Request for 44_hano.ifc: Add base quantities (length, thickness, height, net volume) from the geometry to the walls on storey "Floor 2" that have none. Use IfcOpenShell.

First a look at what the model holds.

```python
import ifcopenshell
import ifcopenshell.util.element
import ifcopenshell.util.unit

model = ifcopenshell.open("44_hano.ifc")
print(model.schema)
for unit_type in ("LENGTHUNIT", "AREAUNIT", "VOLUMEUNIT"):
    print(unit_type, ifcopenshell.util.unit.calculate_unit_scale(model, unit_type))
storey = next(s for s in model.by_type("IfcBuildingStorey") if s.Name == "Floor 2")
walls = [e for e in ifcopenshell.util.element.get_decomposition(storey) if e.is_a("IfcWall")]
for e in sorted(walls, key=lambda e: e.id()):
    print(e.id(), e.is_a(), e.Name, list(ifcopenshell.util.element.get_psets(e, qtos_only=True)), sep=" | ")
```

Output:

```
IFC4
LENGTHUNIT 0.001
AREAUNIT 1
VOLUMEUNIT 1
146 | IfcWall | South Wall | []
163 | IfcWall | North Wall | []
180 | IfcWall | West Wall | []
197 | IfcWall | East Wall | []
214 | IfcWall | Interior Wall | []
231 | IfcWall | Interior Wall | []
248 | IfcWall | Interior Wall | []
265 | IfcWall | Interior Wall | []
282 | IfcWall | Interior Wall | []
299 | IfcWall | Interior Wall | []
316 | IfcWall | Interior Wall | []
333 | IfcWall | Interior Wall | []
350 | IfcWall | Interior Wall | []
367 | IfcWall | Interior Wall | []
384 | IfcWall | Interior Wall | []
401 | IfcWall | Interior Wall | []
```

```python
import ifcopenshell
import ifcopenshell.api.pset
import ifcopenshell.geom
import ifcopenshell.util.element
import ifcopenshell.util.shape
import ifcopenshell.util.unit

model = ifcopenshell.open("44_hano.ifc")
unit_scale = ifcopenshell.util.unit.calculate_unit_scale(model)
volume_scale = ifcopenshell.util.unit.calculate_unit_scale(model, "VOLUMEUNIT")
settings = ifcopenshell.geom.settings()

storey = next(s for s in model.by_type("IfcBuildingStorey") if s.Name == "Floor 2")
walls = [e for e in ifcopenshell.util.element.get_decomposition(storey) if e.is_a("IfcWall")]

for e in sorted(walls, key=lambda e: e.id()):
    if ifcopenshell.util.element.get_psets(e, qtos_only=True, should_inherit=False):
        continue
    # Geometry comes back in metres, in the element's own axes.
    shape = ifcopenshell.geom.create_shape(settings, e)
    values = {
        "Length": ifcopenshell.util.shape.get_x(shape.geometry) / unit_scale,
        "Width": ifcopenshell.util.shape.get_y(shape.geometry) / unit_scale,
        "Height": ifcopenshell.util.shape.get_z(shape.geometry) / unit_scale,
        "NetVolume": ifcopenshell.util.shape.get_volume(shape.geometry) / volume_scale,
    }
    qto = ifcopenshell.api.pset.add_qto(model, product=e, name="Qto_WallBaseQuantities")
    ifcopenshell.api.pset.edit_qto(model, qto=qto, properties=values)
    print(e.id(), {k: round(v, 3) for k, v in values.items()})

model.write("44_hano_v2.ifc")
```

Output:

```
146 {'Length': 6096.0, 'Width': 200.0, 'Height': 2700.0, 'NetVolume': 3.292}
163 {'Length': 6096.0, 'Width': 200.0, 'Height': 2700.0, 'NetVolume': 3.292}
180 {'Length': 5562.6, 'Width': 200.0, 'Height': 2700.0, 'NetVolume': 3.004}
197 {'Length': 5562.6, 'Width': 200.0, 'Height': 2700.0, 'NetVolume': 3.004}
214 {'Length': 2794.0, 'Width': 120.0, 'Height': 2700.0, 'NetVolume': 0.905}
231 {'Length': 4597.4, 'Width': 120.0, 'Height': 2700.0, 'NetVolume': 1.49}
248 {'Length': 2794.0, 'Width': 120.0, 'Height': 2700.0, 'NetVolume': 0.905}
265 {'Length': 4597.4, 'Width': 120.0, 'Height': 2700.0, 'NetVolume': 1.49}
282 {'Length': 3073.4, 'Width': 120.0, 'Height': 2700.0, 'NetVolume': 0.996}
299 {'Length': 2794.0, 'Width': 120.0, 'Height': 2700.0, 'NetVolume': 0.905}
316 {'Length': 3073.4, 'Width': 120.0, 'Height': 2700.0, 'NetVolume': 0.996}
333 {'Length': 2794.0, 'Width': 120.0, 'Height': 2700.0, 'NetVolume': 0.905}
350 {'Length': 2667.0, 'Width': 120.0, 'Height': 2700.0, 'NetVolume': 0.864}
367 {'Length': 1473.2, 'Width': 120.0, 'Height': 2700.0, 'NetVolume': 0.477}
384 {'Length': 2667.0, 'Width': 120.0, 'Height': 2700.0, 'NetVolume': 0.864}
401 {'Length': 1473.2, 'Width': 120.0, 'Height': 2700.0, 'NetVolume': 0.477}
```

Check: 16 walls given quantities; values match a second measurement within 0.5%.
